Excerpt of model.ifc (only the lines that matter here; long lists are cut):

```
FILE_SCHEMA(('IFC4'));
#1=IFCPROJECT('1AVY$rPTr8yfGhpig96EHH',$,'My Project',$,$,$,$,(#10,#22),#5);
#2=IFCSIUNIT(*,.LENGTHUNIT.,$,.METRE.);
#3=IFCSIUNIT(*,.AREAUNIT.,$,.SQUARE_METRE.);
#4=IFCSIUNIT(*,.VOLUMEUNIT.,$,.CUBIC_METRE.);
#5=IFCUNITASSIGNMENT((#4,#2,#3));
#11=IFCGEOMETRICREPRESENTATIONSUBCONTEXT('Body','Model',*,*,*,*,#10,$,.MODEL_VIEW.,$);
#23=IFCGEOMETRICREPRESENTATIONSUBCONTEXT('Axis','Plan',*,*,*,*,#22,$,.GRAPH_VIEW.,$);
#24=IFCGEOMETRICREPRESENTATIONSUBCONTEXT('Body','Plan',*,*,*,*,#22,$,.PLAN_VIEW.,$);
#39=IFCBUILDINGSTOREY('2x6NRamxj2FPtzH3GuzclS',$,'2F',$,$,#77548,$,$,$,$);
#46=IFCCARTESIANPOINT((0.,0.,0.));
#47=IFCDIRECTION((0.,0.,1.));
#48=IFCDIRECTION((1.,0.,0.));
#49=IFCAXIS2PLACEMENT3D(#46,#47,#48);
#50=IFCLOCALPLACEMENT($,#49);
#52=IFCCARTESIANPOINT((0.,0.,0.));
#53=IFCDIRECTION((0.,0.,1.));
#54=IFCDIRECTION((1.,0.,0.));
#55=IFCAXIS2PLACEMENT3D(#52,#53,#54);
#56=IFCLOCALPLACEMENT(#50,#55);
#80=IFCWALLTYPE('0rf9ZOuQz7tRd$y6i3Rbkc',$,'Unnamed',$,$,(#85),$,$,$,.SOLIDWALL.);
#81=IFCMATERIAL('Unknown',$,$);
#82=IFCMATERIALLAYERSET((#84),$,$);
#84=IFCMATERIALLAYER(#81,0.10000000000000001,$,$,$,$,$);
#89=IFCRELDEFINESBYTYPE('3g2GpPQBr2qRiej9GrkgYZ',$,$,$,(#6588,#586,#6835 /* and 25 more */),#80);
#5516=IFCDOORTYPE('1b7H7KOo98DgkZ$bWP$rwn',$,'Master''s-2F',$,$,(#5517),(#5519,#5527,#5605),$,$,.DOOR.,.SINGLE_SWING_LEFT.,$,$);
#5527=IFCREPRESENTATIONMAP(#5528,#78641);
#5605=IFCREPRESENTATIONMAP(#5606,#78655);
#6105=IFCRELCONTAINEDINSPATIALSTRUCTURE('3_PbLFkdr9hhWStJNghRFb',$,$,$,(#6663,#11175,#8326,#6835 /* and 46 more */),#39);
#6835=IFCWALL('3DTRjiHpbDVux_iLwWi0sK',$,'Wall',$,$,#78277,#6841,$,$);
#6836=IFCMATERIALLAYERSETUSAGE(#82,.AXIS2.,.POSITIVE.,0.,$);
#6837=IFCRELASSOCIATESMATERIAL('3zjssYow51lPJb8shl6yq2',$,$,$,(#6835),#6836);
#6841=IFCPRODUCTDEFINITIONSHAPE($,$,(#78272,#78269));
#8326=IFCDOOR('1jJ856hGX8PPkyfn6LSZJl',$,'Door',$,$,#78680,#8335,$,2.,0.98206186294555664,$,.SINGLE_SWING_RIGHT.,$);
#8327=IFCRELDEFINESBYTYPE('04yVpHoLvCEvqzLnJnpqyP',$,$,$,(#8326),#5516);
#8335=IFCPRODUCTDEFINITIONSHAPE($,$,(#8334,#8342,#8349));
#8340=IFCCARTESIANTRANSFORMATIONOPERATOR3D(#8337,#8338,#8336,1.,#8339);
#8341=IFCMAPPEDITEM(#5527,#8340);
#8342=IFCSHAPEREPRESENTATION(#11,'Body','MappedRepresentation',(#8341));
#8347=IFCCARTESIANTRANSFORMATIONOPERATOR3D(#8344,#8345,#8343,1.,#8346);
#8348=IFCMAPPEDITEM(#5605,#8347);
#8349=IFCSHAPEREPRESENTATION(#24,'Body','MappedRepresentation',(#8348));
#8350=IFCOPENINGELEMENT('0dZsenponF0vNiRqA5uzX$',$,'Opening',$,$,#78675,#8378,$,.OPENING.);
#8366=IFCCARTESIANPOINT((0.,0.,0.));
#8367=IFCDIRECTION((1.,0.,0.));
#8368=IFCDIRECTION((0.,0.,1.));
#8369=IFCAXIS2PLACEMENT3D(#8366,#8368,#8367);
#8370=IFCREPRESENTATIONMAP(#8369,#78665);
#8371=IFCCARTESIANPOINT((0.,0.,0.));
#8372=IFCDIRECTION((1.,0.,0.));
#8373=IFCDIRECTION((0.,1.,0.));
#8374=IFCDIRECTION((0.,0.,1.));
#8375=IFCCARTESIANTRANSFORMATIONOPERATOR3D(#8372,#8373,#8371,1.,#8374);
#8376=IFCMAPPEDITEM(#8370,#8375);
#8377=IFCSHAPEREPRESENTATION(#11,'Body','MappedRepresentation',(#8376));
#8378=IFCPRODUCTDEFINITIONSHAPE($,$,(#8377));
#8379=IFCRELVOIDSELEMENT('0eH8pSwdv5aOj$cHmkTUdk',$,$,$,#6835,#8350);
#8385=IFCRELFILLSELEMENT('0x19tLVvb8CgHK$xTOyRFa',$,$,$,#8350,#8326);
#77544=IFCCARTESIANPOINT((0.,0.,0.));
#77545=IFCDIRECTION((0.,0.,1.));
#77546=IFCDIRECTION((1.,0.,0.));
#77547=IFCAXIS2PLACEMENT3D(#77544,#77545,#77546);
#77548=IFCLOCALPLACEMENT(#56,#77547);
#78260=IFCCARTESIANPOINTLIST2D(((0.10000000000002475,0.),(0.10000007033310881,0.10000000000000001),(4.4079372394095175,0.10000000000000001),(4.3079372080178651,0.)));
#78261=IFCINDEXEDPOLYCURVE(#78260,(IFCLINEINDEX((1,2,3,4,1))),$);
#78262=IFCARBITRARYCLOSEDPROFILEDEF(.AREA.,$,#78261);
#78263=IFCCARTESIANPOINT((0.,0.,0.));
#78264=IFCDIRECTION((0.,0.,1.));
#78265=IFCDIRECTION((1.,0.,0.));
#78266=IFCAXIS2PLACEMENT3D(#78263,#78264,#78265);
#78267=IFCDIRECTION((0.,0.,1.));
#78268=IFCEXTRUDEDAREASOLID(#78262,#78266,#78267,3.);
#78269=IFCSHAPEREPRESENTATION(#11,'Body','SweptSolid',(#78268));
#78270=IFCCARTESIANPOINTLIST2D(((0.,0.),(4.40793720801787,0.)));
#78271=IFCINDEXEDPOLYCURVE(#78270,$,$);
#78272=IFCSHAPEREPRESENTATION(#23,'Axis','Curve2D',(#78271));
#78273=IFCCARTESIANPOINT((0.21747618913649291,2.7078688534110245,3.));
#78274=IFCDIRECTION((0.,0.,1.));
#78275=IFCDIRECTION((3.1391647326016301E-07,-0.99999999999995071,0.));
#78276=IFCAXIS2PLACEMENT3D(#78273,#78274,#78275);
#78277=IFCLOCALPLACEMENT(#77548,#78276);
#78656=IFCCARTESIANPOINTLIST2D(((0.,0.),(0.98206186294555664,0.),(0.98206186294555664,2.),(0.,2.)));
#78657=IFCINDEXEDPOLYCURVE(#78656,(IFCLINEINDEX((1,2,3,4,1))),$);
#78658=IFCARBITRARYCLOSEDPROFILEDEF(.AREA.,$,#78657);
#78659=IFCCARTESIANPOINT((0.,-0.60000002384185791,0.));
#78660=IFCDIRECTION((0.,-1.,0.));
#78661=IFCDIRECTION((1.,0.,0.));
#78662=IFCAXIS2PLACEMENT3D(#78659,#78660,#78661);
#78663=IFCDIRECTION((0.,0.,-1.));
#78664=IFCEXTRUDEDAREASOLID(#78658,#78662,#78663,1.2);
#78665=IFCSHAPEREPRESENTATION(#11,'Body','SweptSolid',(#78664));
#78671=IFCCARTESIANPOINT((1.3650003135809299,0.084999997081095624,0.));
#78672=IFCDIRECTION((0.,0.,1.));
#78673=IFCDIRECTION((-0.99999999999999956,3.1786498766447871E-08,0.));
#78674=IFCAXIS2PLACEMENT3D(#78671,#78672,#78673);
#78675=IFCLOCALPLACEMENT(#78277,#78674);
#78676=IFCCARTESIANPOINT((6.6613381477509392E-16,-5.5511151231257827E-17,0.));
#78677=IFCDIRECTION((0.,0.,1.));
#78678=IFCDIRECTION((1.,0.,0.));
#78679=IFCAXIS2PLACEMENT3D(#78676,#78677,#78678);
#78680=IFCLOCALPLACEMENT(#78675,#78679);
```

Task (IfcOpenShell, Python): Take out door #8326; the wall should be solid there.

```python
import ifcopenshell
import ifcopenshell.api.feature
import ifcopenshell.api.root
import ifcopenshell.geom
import ifcopenshell.util.shape

model = ifcopenshell.open("model.ifc")
settings = ifcopenshell.geom.settings()


def volume(element):
    """Net volume in cubic metres, openings subtracted."""
    shape = ifcopenshell.geom.create_shape(settings, element)
    return ifcopenshell.util.shape.get_volume(shape.geometry)


door = model.by_guid("1jJ856hGX8PPkyfn6LSZJl")
opening = door.FillsVoids[0].RelatingOpeningElement
wall = opening.VoidsElements[0].RelatingBuildingElement
before = volume(wall)

ifcopenshell.api.root.remove_product(model, product=door)
ifcopenshell.api.feature.remove_feature(model, feature=opening)

after = volume(wall)

print(f"wall volume {before:.3f} -> {after:.3f} m3")

model.write("model_rev.ifc")
```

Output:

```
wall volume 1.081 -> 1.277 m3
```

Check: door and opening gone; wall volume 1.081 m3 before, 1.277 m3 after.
